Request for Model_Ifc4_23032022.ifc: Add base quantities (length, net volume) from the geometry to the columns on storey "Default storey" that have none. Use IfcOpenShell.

First a look at what the model holds.

```python
import ifcopenshell
import ifcopenshell.util.element
import ifcopenshell.util.unit

model = ifcopenshell.open("Model_Ifc4_23032022.ifc")
print(model.schema)
for unit_type in ("LENGTHUNIT", "AREAUNIT", "VOLUMEUNIT"):
    print(unit_type, ifcopenshell.util.unit.calculate_unit_scale(model, unit_type))
storey = next(s for s in model.by_type("IfcBuildingStorey") if s.Name == "Default storey")
columns = [e for e in ifcopenshell.util.element.get_decomposition(storey) if e.is_a("IfcColumn")]
for e in sorted(columns, key=lambda e: e.id()):
    print(e.id(), e.is_a(), e.Name, list(ifcopenshell.util.element.get_psets(e, qtos_only=True)), sep=" | ")
```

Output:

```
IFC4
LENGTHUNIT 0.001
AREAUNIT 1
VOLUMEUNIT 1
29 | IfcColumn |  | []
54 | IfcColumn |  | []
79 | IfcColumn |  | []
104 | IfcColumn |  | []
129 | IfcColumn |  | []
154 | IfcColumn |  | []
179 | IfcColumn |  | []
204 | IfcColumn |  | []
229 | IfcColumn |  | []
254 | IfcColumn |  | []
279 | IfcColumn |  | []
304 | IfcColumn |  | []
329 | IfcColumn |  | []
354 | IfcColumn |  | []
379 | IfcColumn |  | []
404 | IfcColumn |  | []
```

```python
import ifcopenshell
import ifcopenshell.api.pset
import ifcopenshell.geom
import ifcopenshell.util.element
import ifcopenshell.util.shape
import ifcopenshell.util.unit

model = ifcopenshell.open("Model_Ifc4_23032022.ifc")
unit_scale = ifcopenshell.util.unit.calculate_unit_scale(model)
volume_scale = ifcopenshell.util.unit.calculate_unit_scale(model, "VOLUMEUNIT")
settings = ifcopenshell.geom.settings()

storey = next(s for s in model.by_type("IfcBuildingStorey") if s.Name == "Default storey")
columns = [e for e in ifcopenshell.util.element.get_decomposition(storey) if e.is_a("IfcColumn")]

for e in sorted(columns, key=lambda e: e.id()):
    if ifcopenshell.util.element.get_psets(e, qtos_only=True, should_inherit=False):
        continue
    # Geometry comes back in metres, in the element's own axes.
    shape = ifcopenshell.geom.create_shape(settings, e)
    values = {
        "Length": ifcopenshell.util.shape.get_z(shape.geometry) / unit_scale,
        "NetVolume": ifcopenshell.util.shape.get_volume(shape.geometry) / volume_scale,
    }
    qto = ifcopenshell.api.pset.add_qto(model, product=e, name="Qto_ColumnBaseQuantities")
    ifcopenshell.api.pset.edit_qto(model, qto=qto, properties=values)
    print(e.id(), {k: round(v, 3) for k, v in values.items()})

model.write("Model_Ifc4_23032022_rev.ifc")
```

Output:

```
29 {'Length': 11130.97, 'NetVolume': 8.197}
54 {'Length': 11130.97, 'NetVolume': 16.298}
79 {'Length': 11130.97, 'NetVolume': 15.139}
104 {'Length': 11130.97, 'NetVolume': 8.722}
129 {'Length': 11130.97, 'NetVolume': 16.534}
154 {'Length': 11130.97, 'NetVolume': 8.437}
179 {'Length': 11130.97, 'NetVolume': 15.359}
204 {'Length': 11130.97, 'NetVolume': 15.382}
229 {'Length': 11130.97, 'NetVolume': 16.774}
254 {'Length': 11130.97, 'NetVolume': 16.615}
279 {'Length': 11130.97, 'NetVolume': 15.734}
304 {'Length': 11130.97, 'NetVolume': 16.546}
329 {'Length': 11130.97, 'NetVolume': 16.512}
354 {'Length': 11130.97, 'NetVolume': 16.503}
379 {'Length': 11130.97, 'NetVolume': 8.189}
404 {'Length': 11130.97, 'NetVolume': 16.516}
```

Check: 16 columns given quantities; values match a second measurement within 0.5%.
